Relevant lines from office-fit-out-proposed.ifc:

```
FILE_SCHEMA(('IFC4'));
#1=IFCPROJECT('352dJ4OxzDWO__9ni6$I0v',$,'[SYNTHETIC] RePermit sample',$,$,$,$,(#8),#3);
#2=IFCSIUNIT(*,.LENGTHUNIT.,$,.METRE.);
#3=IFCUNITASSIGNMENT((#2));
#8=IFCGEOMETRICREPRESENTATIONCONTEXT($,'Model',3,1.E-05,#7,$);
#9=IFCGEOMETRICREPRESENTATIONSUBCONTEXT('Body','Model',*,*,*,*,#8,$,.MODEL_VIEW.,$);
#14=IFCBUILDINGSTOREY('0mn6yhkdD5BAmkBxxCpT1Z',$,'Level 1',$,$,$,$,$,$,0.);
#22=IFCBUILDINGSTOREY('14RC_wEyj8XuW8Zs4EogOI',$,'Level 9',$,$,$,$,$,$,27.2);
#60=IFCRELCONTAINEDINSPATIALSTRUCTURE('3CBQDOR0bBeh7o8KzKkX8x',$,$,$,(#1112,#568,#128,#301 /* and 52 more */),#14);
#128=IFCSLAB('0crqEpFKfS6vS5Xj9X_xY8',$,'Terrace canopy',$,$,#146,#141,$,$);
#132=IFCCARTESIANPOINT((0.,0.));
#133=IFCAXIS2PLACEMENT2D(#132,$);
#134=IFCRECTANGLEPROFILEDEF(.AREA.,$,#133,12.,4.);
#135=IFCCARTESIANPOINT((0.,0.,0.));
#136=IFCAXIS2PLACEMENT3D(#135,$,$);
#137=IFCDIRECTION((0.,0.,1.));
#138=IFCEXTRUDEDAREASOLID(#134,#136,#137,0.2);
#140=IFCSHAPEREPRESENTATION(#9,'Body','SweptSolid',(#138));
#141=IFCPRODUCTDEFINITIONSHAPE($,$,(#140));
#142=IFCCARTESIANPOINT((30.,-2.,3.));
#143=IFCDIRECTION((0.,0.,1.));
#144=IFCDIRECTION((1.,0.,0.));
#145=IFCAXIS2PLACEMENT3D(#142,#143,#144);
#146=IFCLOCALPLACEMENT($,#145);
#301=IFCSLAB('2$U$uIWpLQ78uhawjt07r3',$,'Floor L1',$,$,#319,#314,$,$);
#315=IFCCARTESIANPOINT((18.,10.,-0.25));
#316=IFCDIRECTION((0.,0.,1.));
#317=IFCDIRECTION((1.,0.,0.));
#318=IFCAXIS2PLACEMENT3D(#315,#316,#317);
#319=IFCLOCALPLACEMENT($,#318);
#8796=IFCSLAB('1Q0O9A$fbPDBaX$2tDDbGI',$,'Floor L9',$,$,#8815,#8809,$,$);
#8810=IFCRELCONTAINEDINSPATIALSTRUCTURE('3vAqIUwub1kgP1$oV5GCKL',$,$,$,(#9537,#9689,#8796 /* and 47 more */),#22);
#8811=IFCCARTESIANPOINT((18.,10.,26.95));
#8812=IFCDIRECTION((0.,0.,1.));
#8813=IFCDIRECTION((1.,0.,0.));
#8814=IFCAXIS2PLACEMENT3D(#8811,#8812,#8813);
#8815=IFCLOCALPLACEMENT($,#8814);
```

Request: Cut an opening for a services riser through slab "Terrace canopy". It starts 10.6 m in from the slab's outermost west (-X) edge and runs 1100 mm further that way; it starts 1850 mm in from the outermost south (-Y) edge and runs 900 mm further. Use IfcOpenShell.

```python
import numpy as np
import ifcopenshell
import ifcopenshell.api.feature
import ifcopenshell.api.geometry
import ifcopenshell.api.root
import ifcopenshell.geom
import ifcopenshell.util.placement
import ifcopenshell.util.representation
import ifcopenshell.util.shape
import ifcopenshell.util.unit

model = ifcopenshell.open("office-fit-out-proposed.ifc")
unit_scale = ifcopenshell.util.unit.calculate_unit_scale(model)
settings = ifcopenshell.geom.settings()


def volume(element):
    """Net volume in cubic metres, openings subtracted."""
    shape = ifcopenshell.geom.create_shape(settings, element)
    return ifcopenshell.util.shape.get_volume(shape.geometry)


slab = model.by_guid("0crqEpFKfS6vS5Xj9X_xY8")
before = volume(slab)

# Extent in the slab's own axes, in metres. The edges named are its -X and -Y sides.
slab_shape = ifcopenshell.geom.create_shape(settings, slab)
vertices = ifcopenshell.util.shape.get_vertices(slab_shape.geometry)
x_min, y_min, bottom = vertices.min(axis=0)
top = vertices[:, 2].max()

opening = ifcopenshell.api.root.create_entity(model, ifc_class="IfcOpeningElement", name="Services riser opening", predefined_type="OPENING")
context = ifcopenshell.util.representation.get_context(model, "Model", "Body", "MODEL_VIEW")
width, depth = 1.1, 0.9
outline = [(0.0, 0.0), (width, 0.0), (width, depth), (0.0, depth), (0.0, 0.0)]
# Overshoot both faces by 50 mm so the cut is clean.
shape = ifcopenshell.api.geometry.add_slab_representation(
    model, context=context, depth=top - bottom + 0.1, polyline=outline
)
ifcopenshell.api.geometry.assign_representation(model, product=opening, representation=shape)

matrix = ifcopenshell.util.placement.get_local_placement(slab.ObjectPlacement)
matrix[:, 3] = matrix @ np.append(np.array([x_min + 10.6, y_min + 1.85, bottom - 0.05]) / unit_scale, 1.0)
ifcopenshell.api.geometry.edit_object_placement(model, product=opening, matrix=matrix, is_si=False)
ifcopenshell.api.feature.add_feature(model, feature=opening, element=slab)

after = volume(slab)

print(f"slab volume {before:.3f} -> {after:.3f} m3")

model.write("office-fit-out-proposed_rev.ifc")
```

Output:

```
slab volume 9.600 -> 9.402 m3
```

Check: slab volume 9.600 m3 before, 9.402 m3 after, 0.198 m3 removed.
